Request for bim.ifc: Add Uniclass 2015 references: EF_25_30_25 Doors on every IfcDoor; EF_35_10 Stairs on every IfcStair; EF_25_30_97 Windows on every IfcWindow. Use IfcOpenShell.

First a look at what the model holds.

```python
import ifcopenshell

model = ifcopenshell.open("bim.ifc")
print(model.schema)
print("classifications:", [c.Name for c in model.by_type("IfcClassification")])
for ifc_class in ("IfcDoor", "IfcRoof", "IfcStair", "IfcWall", "IfcWindow"):
    print(ifc_class, len(model.by_type(ifc_class)))
```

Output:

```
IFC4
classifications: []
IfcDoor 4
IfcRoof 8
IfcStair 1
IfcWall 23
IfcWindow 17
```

```python
import ifcopenshell
import ifcopenshell.api.classification

model = ifcopenshell.open("bim.ifc")

system = ifcopenshell.api.classification.add_classification(model, classification="Uniclass 2015")

codes = {
    "IfcDoor": ("EF_25_30_25", "Doors"),
    "IfcStair": ("EF_35_10", "Stairs"),
    "IfcWindow": ("EF_25_30_97", "Windows"),
}
for ifc_class, (code, name) in codes.items():
    products = model.by_type(ifc_class)
    ifcopenshell.api.classification.add_reference(
        model, products=products, classification=system, identification=code, name=name
    )
    print(code, len(products))

model.write("bim_v2.ifc")
```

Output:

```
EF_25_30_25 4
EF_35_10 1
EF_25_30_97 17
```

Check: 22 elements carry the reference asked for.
